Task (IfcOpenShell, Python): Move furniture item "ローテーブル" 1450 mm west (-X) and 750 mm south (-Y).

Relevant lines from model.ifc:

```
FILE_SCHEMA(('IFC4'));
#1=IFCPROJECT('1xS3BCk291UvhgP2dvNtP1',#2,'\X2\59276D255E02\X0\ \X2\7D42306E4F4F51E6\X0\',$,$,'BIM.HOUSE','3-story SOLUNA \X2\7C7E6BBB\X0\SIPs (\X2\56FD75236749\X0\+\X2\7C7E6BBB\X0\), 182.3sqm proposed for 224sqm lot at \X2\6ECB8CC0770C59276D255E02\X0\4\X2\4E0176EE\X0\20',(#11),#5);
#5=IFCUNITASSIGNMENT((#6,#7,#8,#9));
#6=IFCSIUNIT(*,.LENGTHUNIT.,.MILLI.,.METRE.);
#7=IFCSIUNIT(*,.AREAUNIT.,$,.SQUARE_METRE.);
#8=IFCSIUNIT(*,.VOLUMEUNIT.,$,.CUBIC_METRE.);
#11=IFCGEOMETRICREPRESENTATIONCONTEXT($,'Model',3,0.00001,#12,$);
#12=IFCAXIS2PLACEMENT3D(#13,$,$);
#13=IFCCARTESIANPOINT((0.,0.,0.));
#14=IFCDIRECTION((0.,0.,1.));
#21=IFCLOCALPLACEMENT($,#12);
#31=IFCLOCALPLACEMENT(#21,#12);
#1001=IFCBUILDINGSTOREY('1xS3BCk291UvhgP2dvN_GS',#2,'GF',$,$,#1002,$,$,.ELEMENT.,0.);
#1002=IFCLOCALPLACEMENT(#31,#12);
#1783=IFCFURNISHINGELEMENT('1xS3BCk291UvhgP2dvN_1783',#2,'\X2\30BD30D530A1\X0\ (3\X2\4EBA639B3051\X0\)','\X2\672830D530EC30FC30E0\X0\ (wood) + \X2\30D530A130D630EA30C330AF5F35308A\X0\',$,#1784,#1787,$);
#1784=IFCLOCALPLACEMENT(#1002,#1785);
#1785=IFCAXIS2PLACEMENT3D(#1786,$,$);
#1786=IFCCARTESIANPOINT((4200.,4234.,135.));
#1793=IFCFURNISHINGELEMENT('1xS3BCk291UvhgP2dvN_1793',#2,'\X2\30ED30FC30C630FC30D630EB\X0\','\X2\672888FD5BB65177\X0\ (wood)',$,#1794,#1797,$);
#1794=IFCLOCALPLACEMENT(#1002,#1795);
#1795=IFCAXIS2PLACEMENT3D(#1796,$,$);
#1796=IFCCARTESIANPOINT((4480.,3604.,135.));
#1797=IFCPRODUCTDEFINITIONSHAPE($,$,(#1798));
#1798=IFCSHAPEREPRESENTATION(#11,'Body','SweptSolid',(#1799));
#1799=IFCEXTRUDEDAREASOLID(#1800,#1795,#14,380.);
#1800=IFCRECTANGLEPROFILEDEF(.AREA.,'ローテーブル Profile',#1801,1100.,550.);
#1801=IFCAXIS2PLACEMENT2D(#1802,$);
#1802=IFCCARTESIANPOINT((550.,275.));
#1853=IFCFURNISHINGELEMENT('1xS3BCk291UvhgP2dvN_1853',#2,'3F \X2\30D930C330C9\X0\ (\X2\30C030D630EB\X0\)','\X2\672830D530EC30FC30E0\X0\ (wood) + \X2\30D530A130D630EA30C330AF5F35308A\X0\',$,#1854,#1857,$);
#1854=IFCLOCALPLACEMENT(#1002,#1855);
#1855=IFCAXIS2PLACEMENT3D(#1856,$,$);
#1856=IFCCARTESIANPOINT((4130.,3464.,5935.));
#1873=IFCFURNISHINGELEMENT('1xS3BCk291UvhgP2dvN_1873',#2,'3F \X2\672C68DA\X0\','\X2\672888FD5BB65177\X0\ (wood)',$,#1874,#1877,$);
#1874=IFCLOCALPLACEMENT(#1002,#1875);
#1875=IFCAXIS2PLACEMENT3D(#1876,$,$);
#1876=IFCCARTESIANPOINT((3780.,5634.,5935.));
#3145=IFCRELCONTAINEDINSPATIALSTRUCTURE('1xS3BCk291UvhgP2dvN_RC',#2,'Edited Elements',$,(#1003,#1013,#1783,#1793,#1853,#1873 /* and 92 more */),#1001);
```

```python
import ifcopenshell
import ifcopenshell.api.geometry
import ifcopenshell.util.placement
import ifcopenshell.util.unit

model = ifcopenshell.open("model.ifc")
unit_scale = ifcopenshell.util.unit.calculate_unit_scale(model)

item = model.by_id(1793)
matrix = ifcopenshell.util.placement.get_local_placement(item.ObjectPlacement)
matrix[0, 3] -= 1.45 / unit_scale
matrix[1, 3] -= 0.75 / unit_scale
ifcopenshell.api.geometry.edit_object_placement(model, product=item, matrix=matrix, is_si=False)

print(ifcopenshell.util.placement.get_local_placement(item.ObjectPlacement).round(3) + 0.0)

model.write("model_v2.ifc")
```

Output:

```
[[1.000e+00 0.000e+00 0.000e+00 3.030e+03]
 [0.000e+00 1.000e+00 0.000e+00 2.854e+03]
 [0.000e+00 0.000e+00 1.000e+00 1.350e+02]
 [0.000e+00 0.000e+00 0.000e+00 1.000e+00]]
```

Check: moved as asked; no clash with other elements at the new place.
